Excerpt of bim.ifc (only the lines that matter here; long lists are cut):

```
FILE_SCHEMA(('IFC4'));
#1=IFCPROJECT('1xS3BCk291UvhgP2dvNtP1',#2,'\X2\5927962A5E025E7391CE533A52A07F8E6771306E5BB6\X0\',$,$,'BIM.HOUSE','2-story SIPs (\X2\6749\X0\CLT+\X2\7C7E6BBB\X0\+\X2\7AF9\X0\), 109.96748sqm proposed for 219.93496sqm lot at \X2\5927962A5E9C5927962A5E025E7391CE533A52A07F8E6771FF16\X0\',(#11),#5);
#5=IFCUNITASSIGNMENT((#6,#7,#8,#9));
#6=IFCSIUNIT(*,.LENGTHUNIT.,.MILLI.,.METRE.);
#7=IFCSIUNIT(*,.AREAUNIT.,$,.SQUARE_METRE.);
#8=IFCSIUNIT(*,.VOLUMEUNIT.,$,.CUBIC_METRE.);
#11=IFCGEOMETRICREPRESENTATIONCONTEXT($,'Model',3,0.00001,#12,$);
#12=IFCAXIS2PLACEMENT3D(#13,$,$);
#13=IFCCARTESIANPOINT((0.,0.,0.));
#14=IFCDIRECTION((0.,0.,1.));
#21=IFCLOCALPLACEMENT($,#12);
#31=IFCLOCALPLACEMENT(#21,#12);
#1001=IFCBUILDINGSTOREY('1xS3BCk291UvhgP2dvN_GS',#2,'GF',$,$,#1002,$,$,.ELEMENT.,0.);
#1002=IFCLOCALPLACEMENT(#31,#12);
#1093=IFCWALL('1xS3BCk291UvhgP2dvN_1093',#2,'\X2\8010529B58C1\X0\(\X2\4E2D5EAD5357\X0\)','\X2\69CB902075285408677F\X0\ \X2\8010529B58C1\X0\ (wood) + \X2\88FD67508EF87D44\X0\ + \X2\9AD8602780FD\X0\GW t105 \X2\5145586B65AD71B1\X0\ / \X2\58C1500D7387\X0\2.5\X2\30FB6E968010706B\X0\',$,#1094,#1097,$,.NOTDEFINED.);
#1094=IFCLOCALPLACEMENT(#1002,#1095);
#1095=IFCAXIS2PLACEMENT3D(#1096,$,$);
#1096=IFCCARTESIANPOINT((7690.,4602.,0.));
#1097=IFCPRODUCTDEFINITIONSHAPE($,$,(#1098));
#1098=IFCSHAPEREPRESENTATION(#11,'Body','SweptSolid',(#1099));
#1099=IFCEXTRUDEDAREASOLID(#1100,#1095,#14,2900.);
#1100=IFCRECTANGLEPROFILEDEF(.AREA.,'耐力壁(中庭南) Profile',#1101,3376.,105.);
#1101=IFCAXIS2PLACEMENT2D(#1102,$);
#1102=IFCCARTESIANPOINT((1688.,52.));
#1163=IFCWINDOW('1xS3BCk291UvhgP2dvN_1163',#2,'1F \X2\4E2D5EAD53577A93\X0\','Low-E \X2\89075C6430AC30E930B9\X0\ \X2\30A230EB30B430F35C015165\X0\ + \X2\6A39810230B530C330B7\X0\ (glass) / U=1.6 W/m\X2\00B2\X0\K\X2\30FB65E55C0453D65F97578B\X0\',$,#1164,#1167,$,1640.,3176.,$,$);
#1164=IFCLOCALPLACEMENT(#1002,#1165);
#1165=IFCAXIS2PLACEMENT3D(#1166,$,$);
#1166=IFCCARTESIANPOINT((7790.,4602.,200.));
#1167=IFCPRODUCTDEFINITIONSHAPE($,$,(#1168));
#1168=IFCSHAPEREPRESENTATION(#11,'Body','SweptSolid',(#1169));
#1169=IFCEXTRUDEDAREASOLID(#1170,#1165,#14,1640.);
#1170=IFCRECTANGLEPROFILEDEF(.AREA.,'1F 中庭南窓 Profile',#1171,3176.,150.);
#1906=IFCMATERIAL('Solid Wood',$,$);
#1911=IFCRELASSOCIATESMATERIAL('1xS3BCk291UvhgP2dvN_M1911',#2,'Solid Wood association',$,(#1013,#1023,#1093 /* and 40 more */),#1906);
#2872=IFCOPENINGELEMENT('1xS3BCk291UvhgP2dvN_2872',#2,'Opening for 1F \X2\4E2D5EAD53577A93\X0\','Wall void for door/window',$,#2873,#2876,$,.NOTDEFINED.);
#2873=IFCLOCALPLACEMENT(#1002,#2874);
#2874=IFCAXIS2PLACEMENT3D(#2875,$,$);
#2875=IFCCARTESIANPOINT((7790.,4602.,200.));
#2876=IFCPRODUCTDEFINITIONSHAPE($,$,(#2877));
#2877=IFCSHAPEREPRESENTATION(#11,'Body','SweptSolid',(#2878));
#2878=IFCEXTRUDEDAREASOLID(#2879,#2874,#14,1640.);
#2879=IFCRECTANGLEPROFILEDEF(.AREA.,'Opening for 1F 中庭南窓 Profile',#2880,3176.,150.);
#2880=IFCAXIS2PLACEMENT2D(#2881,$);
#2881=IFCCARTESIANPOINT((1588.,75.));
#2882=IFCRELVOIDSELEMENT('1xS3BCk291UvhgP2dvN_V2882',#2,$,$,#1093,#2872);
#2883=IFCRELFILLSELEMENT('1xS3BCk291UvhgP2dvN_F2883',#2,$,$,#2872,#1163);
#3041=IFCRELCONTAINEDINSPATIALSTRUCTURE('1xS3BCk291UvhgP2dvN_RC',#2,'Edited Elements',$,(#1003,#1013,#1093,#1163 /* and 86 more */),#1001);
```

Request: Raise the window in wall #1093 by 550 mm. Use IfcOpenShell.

```python
import numpy as np
import ifcopenshell
import ifcopenshell.api.geometry
import ifcopenshell.util.placement
import ifcopenshell.util.unit

model = ifcopenshell.open("bim.ifc")
unit_scale = ifcopenshell.util.unit.calculate_unit_scale(model)

window = model.by_id(1163)
opening = window.FillsVoids[0].RelatingOpeningElement
dz = 0.55 / unit_scale

shift = np.array([0.0, 0.0, dz])
# The window is not placed relative to its opening, so move both.
for product in (opening, window):
    matrix = ifcopenshell.util.placement.get_local_placement(product.ObjectPlacement)
    matrix[:3, 3] += shift
    ifcopenshell.api.geometry.edit_object_placement(model, product=product, matrix=matrix, is_si=False)

print(f"moved by {dz * unit_scale:+.3f} m")

model.write("bim-out.ifc")
```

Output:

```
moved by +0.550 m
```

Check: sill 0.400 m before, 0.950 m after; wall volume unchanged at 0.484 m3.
